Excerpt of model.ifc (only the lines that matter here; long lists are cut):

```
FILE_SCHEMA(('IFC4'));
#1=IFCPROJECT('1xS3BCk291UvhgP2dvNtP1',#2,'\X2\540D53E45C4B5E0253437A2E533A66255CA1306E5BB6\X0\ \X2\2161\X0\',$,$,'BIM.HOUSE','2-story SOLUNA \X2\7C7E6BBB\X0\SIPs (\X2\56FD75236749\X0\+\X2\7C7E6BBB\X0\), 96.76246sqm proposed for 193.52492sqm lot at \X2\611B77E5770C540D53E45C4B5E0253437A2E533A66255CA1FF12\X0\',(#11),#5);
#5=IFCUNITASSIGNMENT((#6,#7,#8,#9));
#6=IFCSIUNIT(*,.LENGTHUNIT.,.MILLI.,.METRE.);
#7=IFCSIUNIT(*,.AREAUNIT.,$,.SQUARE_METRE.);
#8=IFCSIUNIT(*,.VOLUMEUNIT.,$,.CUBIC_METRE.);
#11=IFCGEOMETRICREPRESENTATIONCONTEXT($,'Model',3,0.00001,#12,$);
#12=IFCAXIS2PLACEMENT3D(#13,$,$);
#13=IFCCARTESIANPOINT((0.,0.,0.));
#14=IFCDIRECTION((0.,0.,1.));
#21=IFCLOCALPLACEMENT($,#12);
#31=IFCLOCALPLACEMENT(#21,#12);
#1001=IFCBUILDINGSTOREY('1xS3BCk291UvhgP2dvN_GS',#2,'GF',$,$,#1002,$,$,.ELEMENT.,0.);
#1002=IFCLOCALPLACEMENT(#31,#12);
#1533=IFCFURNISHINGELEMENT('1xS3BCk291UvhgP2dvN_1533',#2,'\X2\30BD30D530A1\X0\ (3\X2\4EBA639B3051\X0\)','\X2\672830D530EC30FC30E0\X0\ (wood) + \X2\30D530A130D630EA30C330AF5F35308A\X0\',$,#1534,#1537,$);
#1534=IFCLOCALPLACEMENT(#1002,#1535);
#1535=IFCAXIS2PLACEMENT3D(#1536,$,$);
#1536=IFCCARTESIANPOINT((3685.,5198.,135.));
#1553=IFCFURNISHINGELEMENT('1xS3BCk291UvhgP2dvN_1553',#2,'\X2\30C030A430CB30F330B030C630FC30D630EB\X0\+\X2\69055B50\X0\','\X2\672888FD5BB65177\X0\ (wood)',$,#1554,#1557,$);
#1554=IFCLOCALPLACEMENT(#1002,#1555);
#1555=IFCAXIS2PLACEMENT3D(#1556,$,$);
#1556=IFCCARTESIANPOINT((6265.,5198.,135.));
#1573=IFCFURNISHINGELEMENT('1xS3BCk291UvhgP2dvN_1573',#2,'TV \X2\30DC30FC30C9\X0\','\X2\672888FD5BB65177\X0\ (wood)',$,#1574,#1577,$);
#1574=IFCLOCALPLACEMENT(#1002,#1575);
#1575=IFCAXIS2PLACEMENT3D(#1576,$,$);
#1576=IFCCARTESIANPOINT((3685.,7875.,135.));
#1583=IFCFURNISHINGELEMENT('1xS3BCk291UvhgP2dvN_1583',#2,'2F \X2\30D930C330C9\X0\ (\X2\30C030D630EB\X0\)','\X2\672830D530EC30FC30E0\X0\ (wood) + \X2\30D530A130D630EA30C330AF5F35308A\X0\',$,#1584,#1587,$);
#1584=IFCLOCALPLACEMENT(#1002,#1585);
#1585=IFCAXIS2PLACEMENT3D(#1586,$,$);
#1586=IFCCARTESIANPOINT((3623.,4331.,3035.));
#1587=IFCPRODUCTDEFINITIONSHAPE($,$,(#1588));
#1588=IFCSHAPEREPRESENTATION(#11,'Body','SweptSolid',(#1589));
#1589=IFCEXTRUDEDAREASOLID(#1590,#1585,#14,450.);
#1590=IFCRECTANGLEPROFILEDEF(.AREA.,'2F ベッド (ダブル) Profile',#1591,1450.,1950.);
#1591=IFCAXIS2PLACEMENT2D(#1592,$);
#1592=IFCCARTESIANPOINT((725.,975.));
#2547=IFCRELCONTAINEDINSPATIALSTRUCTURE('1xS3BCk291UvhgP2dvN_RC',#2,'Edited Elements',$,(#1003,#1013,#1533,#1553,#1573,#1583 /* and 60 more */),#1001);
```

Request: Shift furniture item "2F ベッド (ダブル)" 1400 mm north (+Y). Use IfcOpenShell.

```python
import ifcopenshell
import ifcopenshell.api.geometry
import ifcopenshell.util.placement
import ifcopenshell.util.unit

model = ifcopenshell.open("model.ifc")
unit_scale = ifcopenshell.util.unit.calculate_unit_scale(model)

item = model.by_guid("1xS3BCk291UvhgP2dvN_1583")
matrix = ifcopenshell.util.placement.get_local_placement(item.ObjectPlacement)
matrix[1, 3] += 1.4 / unit_scale
ifcopenshell.api.geometry.edit_object_placement(model, product=item, matrix=matrix, is_si=False)

print(ifcopenshell.util.placement.get_local_placement(item.ObjectPlacement).round(3) + 0.0)

model.write("model_edited.ifc")
```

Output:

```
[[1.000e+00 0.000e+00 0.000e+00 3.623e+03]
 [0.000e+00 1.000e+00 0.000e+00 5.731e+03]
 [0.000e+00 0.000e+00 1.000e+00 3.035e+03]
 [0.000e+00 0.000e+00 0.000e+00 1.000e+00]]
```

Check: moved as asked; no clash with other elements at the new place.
